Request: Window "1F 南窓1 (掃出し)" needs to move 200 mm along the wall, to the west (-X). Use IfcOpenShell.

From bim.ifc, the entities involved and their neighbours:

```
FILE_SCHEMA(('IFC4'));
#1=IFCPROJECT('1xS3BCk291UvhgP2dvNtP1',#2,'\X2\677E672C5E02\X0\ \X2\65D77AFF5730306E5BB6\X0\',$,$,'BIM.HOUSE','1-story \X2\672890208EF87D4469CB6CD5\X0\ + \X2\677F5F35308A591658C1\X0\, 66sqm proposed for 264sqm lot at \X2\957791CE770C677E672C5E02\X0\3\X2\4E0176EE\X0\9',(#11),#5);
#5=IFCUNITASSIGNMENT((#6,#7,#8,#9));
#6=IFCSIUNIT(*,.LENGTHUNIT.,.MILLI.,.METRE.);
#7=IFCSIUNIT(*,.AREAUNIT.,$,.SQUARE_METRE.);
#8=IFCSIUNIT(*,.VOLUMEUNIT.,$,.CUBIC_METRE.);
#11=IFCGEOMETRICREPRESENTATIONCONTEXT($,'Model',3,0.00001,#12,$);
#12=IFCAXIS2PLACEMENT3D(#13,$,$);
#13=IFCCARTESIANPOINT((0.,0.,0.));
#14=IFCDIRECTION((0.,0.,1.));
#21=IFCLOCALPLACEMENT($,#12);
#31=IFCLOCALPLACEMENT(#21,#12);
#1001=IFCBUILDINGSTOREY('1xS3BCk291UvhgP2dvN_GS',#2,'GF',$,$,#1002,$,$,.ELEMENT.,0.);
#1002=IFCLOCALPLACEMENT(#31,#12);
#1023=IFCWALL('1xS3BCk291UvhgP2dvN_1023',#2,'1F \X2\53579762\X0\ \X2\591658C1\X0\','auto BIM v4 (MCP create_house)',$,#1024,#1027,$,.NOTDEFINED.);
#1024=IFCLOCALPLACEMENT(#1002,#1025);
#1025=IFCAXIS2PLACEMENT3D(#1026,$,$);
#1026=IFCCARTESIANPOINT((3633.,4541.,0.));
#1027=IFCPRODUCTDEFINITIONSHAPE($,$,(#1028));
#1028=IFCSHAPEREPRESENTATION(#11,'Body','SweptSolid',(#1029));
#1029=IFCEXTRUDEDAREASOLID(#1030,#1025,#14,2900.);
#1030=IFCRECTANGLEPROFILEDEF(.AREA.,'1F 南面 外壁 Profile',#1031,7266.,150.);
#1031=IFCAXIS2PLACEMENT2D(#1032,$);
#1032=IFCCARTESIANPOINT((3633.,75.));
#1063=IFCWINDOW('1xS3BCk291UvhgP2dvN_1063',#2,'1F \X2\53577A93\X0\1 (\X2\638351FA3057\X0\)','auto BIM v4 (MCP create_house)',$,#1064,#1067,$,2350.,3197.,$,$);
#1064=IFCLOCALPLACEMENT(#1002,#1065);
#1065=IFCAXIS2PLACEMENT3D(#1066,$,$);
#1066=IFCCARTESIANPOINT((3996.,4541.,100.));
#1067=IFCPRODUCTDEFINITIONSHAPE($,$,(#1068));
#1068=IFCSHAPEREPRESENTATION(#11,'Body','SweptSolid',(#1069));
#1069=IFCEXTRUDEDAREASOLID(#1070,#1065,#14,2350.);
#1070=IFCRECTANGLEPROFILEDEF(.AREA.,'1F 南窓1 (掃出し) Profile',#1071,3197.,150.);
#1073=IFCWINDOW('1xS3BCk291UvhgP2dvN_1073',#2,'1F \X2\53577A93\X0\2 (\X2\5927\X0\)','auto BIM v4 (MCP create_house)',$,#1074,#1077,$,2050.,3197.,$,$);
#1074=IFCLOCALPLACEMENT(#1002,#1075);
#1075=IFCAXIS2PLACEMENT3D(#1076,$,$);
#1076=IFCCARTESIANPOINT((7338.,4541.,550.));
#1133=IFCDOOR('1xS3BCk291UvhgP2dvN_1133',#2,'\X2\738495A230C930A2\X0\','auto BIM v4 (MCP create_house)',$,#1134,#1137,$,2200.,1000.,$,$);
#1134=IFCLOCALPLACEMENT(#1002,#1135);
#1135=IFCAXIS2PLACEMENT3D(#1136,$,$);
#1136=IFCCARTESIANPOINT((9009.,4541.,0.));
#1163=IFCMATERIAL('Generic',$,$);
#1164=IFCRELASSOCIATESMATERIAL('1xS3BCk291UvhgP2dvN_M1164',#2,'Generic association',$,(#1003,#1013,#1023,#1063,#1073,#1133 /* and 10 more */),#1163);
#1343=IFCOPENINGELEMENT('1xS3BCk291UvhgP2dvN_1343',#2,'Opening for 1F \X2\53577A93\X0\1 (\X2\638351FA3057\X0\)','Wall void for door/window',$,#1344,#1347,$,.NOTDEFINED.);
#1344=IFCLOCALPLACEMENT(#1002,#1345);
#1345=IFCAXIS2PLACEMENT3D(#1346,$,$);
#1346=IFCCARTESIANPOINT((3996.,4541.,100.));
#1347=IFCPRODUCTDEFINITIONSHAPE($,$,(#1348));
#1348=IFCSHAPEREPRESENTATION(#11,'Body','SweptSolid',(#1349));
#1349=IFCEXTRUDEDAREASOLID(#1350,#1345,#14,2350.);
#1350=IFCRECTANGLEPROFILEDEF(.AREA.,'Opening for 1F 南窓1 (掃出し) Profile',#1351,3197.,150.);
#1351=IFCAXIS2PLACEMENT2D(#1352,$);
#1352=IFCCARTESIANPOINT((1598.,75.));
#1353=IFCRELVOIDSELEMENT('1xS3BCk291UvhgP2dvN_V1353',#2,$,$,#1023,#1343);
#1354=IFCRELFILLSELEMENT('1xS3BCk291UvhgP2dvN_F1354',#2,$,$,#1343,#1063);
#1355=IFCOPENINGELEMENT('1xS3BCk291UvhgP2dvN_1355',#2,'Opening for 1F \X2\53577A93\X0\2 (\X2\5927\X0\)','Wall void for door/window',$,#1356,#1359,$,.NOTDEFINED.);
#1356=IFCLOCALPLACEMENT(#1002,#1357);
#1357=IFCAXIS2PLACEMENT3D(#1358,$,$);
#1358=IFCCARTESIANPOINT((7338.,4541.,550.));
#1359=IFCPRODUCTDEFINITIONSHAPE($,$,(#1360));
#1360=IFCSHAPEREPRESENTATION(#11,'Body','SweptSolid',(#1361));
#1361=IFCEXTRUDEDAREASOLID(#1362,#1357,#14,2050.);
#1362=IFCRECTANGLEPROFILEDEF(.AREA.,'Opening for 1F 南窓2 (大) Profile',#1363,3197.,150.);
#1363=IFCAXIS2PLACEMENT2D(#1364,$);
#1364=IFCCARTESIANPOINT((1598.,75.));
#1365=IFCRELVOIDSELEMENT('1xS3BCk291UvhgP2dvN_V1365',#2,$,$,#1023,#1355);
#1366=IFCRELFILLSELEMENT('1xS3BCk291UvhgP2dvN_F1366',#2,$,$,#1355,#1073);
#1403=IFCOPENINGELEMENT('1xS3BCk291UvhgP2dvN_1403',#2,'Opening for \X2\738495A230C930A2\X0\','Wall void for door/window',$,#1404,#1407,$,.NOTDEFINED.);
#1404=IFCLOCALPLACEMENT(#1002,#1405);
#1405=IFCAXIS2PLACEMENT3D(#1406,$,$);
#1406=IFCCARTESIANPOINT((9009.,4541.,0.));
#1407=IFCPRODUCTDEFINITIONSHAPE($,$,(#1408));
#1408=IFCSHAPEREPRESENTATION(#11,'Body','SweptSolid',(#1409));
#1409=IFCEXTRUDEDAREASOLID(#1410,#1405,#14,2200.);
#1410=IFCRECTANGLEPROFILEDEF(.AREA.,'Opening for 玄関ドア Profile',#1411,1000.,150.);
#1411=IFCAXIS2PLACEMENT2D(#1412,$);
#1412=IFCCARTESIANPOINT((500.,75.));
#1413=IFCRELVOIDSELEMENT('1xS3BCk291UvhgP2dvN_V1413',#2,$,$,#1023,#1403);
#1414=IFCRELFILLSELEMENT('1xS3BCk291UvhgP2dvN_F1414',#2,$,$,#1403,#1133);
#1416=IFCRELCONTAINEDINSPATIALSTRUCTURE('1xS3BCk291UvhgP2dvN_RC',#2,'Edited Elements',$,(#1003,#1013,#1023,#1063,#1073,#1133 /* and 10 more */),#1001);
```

```python
import ifcopenshell
import ifcopenshell.api.geometry
import ifcopenshell.util.placement
import ifcopenshell.util.unit

model = ifcopenshell.open("bim.ifc")
unit_scale = ifcopenshell.util.unit.calculate_unit_scale(model)

window = model.by_guid("1xS3BCk291UvhgP2dvN_1063")
opening = window.FillsVoids[0].RelatingOpeningElement
wall = opening.VoidsElements[0].RelatingBuildingElement

wall_matrix = ifcopenshell.util.placement.get_local_placement(wall.ObjectPlacement)
shift = wall_matrix[:3, 0] * -0.2 / unit_scale
before = ifcopenshell.util.placement.get_local_placement(window.ObjectPlacement)[:3, 3].copy()

# The window is not placed relative to its opening, so move both.
for product in (opening, window):
    matrix = ifcopenshell.util.placement.get_local_placement(product.ObjectPlacement)
    matrix[:3, 3] += shift
    ifcopenshell.api.geometry.edit_object_placement(model, product=product, matrix=matrix, is_si=False)

after = ifcopenshell.util.placement.get_local_placement(window.ObjectPlacement)[:3, 3]
print("window moved by", (after - before).round(3) + 0.0)

model.write("bim_edited.ifc")
```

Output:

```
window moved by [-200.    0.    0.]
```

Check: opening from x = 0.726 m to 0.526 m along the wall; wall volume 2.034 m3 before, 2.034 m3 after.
